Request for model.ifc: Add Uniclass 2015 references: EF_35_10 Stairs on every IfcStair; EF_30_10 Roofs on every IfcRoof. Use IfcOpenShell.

First a look at what the model holds.

```python
import ifcopenshell

model = ifcopenshell.open("model.ifc")
print(model.schema)
print("classifications:", [c.Name for c in model.by_type("IfcClassification")])
for ifc_class in ("IfcDoor", "IfcRoof", "IfcStair", "IfcWall", "IfcWindow"):
    print(ifc_class, len(model.by_type(ifc_class)))
```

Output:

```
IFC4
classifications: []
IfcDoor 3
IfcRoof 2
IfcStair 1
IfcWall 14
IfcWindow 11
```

```python
import ifcopenshell
import ifcopenshell.api.classification

model = ifcopenshell.open("model.ifc")

system = ifcopenshell.api.classification.add_classification(model, classification="Uniclass 2015")

codes = {
    "IfcStair": ("EF_35_10", "Stairs"),
    "IfcRoof": ("EF_30_10", "Roofs"),
}
for ifc_class, (code, name) in codes.items():
    products = model.by_type(ifc_class)
    ifcopenshell.api.classification.add_reference(
        model, products=products, classification=system, identification=code, name=name
    )
    print(code, len(products))

model.write("model-out.ifc")
```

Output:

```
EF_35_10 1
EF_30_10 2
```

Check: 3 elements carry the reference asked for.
